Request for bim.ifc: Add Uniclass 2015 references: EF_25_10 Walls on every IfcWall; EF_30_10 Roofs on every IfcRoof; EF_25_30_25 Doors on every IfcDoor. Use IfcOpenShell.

First a look at what the model holds.

```python
import ifcopenshell

model = ifcopenshell.open("bim.ifc")
print(model.schema)
print("classifications:", [c.Name for c in model.by_type("IfcClassification")])
for ifc_class in ("IfcDoor", "IfcRoof", "IfcStair", "IfcWall", "IfcWindow"):
    print(ifc_class, len(model.by_type(ifc_class)))
```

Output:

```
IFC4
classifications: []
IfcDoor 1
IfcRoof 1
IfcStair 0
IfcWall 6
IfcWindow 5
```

```python
import ifcopenshell
import ifcopenshell.api.classification

model = ifcopenshell.open("bim.ifc")

system = ifcopenshell.api.classification.add_classification(model, classification="Uniclass 2015")

codes = {
    "IfcWall": ("EF_25_10", "Walls"),
    "IfcRoof": ("EF_30_10", "Roofs"),
    "IfcDoor": ("EF_25_30_25", "Doors"),
}
for ifc_class, (code, name) in codes.items():
    products = model.by_type(ifc_class)
    ifcopenshell.api.classification.add_reference(
        model, products=products, classification=system, identification=code, name=name
    )
    print(code, len(products))

model.write("bim_v2.ifc")
```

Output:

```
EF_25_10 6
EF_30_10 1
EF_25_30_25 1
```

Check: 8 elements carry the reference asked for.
